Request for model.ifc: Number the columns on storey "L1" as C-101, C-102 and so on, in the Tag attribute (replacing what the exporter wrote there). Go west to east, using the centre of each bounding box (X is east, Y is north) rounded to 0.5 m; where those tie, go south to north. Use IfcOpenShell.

First a look at what the model holds.

```python
import ifcopenshell
import ifcopenshell.util.element
import ifcopenshell.util.placement

model = ifcopenshell.open("model.ifc")
print(model.schema)
storey = next(s for s in model.by_type("IfcBuildingStorey") if s.Name == "L1")
columns = [e for e in ifcopenshell.util.element.get_decomposition(storey) if e.is_a("IfcColumn")]
for e in sorted(columns, key=lambda e: e.id()):
    origin = ifcopenshell.util.placement.get_local_placement(e.ObjectPlacement)[:3, 3]
    print(e.id(), e.Tag, e.Name, origin.round(2) + 0.0, sep=" | ")
```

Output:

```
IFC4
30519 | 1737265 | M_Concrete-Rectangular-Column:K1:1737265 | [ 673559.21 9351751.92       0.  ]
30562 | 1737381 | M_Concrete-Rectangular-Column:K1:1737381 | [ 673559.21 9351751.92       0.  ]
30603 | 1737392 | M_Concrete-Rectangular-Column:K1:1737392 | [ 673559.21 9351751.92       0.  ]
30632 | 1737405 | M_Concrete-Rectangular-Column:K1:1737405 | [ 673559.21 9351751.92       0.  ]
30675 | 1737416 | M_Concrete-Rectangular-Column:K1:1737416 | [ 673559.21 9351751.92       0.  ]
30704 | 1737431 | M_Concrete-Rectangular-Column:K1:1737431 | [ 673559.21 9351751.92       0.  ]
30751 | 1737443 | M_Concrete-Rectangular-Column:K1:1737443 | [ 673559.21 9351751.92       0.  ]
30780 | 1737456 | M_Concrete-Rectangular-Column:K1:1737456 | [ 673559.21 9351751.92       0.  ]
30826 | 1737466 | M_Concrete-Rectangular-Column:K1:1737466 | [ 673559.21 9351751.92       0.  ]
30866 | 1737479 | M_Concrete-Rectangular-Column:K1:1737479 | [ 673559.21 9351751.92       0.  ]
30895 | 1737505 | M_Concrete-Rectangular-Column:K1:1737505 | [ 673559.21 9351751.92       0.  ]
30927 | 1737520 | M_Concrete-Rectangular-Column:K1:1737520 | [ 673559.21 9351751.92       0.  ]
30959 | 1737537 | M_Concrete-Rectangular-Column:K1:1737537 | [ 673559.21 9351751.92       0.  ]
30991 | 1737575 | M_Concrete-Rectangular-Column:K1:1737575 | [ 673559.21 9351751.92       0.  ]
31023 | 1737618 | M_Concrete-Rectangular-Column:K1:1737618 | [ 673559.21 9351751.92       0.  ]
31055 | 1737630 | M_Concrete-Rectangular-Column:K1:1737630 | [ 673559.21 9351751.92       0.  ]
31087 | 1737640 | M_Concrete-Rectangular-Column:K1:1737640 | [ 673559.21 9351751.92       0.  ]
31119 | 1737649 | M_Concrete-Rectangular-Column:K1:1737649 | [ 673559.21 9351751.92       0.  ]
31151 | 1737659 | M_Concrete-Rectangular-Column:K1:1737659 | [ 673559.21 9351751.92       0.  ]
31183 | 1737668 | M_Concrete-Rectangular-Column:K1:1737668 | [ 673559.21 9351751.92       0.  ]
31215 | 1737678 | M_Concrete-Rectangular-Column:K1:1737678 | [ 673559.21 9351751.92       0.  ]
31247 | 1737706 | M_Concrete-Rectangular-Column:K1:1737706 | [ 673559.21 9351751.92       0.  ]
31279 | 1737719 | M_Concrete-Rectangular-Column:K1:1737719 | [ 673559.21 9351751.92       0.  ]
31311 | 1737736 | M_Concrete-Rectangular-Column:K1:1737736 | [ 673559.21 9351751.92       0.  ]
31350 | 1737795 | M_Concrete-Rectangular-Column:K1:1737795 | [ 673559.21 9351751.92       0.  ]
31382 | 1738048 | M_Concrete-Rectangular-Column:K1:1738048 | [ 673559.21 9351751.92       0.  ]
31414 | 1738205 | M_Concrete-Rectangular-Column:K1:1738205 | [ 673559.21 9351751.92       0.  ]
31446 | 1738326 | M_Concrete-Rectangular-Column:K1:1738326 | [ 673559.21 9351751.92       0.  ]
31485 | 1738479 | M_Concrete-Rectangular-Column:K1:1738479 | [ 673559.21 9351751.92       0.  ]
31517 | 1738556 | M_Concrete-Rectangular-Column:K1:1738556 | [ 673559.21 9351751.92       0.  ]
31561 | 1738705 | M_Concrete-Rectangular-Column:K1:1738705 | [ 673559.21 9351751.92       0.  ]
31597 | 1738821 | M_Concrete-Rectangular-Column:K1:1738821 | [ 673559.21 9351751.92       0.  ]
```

```python
import ifcopenshell
import ifcopenshell.geom
import ifcopenshell.util.element
import ifcopenshell.util.shape

model = ifcopenshell.open("model.ifc")
settings = ifcopenshell.geom.settings()
settings.set("use-world-coords", True)


def centre(element):
    shape = ifcopenshell.geom.create_shape(settings, element)
    return ifcopenshell.util.shape.get_bbox_centroid(shape.geometry)


storey = next(s for s in model.by_type("IfcBuildingStorey") if s.Name == "L1")
columns = [e for e in ifcopenshell.util.element.get_decomposition(storey) if e.is_a("IfcColumn")]

# Insertion points can sit at a corner or the storey origin, so sort by the geometry (in metres).
centres = {e: centre(e) for e in columns}
columns.sort(key=lambda e: (round(centres[e][0] / 0.5), centres[e][1]))

for i, e in enumerate(columns, start=1):
    number = f"C-1{i:02d}"
    e.Tag = number
    print(e.id(), number)

model.write("model_updated.ifc")
```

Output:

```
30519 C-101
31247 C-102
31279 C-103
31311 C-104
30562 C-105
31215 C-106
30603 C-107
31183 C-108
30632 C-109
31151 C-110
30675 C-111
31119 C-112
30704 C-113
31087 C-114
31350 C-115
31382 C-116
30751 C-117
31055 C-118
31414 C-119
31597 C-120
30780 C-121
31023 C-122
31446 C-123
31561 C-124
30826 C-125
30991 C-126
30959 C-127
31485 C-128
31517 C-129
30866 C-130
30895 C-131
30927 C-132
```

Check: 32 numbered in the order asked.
